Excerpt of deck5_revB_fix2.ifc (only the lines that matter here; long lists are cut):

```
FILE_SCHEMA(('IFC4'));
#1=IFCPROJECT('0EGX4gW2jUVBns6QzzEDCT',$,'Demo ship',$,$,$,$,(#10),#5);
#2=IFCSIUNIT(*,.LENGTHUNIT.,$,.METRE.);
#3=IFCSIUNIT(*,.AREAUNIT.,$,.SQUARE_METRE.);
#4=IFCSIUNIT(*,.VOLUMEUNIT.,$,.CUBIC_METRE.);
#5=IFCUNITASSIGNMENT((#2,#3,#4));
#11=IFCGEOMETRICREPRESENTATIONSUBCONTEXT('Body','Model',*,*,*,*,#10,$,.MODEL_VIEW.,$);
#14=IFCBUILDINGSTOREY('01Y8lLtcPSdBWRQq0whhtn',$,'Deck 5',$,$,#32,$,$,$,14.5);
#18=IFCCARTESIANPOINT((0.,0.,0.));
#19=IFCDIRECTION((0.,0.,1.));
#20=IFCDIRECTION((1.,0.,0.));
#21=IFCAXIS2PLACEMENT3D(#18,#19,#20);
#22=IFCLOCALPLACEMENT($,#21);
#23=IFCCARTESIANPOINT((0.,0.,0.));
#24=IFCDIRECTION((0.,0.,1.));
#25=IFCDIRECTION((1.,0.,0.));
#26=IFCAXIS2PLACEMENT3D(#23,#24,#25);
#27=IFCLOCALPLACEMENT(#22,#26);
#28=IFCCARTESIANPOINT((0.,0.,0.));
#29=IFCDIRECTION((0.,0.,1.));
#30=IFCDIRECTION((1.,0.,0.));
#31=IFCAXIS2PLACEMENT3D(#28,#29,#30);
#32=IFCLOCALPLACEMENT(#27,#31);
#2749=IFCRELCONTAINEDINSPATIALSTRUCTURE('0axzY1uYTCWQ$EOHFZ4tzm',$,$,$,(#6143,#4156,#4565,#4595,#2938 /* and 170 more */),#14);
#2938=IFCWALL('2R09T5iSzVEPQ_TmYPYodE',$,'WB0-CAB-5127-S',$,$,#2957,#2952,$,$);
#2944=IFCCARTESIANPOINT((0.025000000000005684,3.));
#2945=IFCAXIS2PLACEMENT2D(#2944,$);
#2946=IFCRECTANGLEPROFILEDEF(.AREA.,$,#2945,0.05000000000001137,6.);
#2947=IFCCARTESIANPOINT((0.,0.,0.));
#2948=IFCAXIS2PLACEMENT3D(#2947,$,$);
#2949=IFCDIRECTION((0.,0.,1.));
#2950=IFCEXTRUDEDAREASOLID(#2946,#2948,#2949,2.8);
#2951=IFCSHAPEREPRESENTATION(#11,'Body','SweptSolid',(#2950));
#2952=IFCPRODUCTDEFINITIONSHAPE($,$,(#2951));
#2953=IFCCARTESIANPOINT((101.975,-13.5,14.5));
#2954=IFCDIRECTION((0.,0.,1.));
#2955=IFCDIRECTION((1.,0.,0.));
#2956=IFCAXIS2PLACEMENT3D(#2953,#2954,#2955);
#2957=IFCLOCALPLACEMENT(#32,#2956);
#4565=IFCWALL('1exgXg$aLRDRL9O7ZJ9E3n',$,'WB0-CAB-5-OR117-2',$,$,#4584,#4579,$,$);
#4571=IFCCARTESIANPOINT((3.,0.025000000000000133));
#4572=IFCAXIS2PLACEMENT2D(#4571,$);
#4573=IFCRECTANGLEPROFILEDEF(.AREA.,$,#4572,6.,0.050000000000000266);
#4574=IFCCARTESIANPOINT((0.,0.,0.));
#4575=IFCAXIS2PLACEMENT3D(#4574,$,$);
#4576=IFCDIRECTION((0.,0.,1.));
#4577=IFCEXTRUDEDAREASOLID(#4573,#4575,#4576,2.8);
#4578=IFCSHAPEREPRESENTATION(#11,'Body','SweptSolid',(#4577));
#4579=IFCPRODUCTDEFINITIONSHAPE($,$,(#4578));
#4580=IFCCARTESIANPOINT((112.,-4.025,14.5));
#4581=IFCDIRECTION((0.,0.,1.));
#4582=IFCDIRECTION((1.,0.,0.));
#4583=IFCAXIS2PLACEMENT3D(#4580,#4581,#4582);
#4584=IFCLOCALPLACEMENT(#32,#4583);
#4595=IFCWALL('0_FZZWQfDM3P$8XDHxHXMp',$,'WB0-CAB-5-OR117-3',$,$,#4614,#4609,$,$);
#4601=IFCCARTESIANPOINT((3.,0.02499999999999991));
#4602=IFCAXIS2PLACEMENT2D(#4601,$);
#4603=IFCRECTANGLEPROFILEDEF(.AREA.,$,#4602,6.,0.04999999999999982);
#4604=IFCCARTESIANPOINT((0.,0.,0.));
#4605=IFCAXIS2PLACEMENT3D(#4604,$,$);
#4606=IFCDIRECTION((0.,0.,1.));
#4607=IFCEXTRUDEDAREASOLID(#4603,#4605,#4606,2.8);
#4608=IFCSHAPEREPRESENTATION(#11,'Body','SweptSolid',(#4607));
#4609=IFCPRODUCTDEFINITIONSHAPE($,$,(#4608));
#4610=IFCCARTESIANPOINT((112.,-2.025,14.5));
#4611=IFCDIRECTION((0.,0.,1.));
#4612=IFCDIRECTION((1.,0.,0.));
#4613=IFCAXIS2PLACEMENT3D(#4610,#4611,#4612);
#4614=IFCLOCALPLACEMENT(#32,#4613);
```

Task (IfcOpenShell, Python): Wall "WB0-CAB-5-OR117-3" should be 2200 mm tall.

```python
import ifcopenshell
import ifcopenshell.geom
import ifcopenshell.util.representation
import ifcopenshell.util.shape
import ifcopenshell.util.unit

model = ifcopenshell.open("deck5_revB_fix2.ifc")
unit_scale = ifcopenshell.util.unit.calculate_unit_scale(model)
settings = ifcopenshell.geom.settings()


def volume(element):
    """Net volume in cubic metres, openings subtracted."""
    shape = ifcopenshell.geom.create_shape(settings, element)
    return ifcopenshell.util.shape.get_volume(shape.geometry)


wall = model.by_id(4595)
before = volume(wall)

body = ifcopenshell.util.representation.get_representation(wall, "Model", "Body")
solid = body.Items[0]
old_height = solid.Depth
solid.Depth = 2.2 / unit_scale
after = volume(wall)

print(f"height {old_height:g} -> {solid.Depth:g}, volume {before:.3f} -> {after:.3f} m3")

model.write("deck5_revB_fix2_v2.ifc")
```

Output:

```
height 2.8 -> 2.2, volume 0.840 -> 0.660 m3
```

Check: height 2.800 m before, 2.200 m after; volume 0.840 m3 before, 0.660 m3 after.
